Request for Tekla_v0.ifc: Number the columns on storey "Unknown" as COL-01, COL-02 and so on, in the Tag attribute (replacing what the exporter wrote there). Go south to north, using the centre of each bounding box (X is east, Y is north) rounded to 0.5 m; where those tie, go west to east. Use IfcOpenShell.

First a look at what the model holds.

```python
import ifcopenshell
import ifcopenshell.util.element
import ifcopenshell.util.placement

model = ifcopenshell.open("Tekla_v0.ifc")
print(model.schema)
storey = next(s for s in model.by_type("IfcBuildingStorey") if s.Name == "Unknown")
columns = [e for e in ifcopenshell.util.element.get_decomposition(storey) if e.is_a("IfcColumn")]
for e in sorted(columns, key=lambda e: e.id()):
    origin = ifcopenshell.util.placement.get_local_placement(e.ObjectPlacement)[:3, 3]
    print(e.id(), e.Tag, e.Name, origin.round(2) + 0.0, sep=" | ")
```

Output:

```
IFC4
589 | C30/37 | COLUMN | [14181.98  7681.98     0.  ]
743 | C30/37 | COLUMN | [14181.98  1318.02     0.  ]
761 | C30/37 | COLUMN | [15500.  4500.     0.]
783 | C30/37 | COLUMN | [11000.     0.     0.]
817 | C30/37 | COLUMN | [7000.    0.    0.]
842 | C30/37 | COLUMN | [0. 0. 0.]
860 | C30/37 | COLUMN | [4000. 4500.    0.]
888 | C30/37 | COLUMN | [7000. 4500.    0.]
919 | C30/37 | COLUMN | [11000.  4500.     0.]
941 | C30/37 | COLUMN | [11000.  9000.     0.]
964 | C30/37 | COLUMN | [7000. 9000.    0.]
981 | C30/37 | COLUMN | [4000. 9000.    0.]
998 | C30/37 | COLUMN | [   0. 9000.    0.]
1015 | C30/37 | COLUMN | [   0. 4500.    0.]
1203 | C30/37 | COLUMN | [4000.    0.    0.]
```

```python
import ifcopenshell
import ifcopenshell.geom
import ifcopenshell.util.element
import ifcopenshell.util.shape

model = ifcopenshell.open("Tekla_v0.ifc")
settings = ifcopenshell.geom.settings()
settings.set("use-world-coords", True)


def centre(element):
    shape = ifcopenshell.geom.create_shape(settings, element)
    return ifcopenshell.util.shape.get_bbox_centroid(shape.geometry)


storey = next(s for s in model.by_type("IfcBuildingStorey") if s.Name == "Unknown")
columns = [e for e in ifcopenshell.util.element.get_decomposition(storey) if e.is_a("IfcColumn")]

# Insertion points can sit at a corner or the storey origin, so sort by the geometry (in metres).
centres = {e: centre(e) for e in columns}
columns.sort(key=lambda e: (round(centres[e][1] / 0.5), centres[e][0]))

for i, e in enumerate(columns, start=1):
    number = f"COL-{i:02d}"
    e.Tag = number
    print(e.id(), number)

model.write("Tekla_v0_v2.ifc")
```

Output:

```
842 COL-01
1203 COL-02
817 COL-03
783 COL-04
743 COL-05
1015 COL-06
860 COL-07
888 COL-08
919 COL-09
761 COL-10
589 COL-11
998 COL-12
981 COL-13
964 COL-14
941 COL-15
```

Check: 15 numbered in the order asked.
